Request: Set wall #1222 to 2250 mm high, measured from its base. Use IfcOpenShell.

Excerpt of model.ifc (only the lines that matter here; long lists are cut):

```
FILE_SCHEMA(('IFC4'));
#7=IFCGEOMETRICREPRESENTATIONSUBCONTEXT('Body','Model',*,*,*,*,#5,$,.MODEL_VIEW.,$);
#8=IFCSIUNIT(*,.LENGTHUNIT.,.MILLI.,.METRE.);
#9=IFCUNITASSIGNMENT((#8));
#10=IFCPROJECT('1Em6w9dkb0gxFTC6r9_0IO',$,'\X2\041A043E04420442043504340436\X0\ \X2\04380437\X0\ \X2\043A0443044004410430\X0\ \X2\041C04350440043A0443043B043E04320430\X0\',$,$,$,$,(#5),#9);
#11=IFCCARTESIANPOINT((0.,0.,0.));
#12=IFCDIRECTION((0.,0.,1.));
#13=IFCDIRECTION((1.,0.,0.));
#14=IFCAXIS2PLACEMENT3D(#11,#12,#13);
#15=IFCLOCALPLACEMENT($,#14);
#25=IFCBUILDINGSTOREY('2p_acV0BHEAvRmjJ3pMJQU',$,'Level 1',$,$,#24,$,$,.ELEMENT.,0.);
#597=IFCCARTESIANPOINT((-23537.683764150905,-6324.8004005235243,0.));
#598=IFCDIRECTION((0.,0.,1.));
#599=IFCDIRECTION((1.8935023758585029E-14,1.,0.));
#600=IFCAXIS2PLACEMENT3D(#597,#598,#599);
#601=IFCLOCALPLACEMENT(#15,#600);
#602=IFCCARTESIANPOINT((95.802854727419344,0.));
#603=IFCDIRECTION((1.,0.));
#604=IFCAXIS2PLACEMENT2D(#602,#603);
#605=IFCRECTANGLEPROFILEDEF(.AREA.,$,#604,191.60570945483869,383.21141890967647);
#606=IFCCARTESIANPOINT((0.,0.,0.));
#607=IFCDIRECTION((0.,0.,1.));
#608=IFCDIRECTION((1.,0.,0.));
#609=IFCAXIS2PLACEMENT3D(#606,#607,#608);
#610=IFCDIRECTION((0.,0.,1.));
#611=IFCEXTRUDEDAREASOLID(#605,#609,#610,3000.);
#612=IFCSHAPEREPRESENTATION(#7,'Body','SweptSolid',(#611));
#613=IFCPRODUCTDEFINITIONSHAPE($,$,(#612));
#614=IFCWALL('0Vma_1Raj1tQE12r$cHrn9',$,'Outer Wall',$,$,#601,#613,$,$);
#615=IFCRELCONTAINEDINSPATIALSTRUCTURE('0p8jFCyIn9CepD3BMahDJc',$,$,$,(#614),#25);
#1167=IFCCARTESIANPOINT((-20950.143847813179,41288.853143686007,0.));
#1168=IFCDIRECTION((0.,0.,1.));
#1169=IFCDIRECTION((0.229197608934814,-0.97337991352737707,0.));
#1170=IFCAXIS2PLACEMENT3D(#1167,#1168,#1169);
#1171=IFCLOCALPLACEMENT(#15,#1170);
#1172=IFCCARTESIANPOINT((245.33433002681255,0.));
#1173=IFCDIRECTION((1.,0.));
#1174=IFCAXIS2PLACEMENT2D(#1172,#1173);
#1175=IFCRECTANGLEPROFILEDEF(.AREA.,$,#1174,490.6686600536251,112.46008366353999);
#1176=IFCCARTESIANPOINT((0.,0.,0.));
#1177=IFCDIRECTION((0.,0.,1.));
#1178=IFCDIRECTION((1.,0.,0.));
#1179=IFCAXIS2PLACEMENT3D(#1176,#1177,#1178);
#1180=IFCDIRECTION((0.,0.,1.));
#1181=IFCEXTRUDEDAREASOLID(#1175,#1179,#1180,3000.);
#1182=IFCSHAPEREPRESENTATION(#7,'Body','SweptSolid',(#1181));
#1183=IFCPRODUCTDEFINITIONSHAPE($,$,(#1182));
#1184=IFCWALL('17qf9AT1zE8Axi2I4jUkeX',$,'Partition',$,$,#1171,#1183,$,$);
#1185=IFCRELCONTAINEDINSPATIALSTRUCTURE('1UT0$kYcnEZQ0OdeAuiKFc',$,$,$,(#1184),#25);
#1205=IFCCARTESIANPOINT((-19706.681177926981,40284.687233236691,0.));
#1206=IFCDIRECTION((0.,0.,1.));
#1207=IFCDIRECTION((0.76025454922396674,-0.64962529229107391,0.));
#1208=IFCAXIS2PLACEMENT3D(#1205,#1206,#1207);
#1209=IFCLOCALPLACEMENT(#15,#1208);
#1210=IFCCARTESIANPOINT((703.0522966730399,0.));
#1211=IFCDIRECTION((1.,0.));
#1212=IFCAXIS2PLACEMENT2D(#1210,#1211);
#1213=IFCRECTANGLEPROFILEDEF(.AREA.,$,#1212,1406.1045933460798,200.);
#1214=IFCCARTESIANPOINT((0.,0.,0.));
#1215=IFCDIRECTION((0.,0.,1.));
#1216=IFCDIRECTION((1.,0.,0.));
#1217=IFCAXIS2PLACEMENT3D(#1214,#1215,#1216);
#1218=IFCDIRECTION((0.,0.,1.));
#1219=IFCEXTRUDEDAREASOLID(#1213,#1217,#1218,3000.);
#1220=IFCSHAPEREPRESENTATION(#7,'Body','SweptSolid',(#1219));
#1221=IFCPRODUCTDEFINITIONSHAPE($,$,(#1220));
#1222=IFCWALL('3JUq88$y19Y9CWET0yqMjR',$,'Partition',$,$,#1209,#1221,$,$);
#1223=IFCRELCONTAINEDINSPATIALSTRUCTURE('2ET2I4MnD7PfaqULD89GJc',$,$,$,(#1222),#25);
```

```python
import ifcopenshell
import ifcopenshell.geom
import ifcopenshell.util.representation
import ifcopenshell.util.shape
import ifcopenshell.util.unit

model = ifcopenshell.open("model.ifc")
unit_scale = ifcopenshell.util.unit.calculate_unit_scale(model)
settings = ifcopenshell.geom.settings()


def volume(element):
    """Net volume in cubic metres, openings subtracted."""
    shape = ifcopenshell.geom.create_shape(settings, element)
    return ifcopenshell.util.shape.get_volume(shape.geometry)


wall = model.by_guid("3JUq88$y19Y9CWET0yqMjR")
before = volume(wall)

body = ifcopenshell.util.representation.get_representation(wall, "Model", "Body")
solid = body.Items[0]
old_height = solid.Depth
solid.Depth = 2.25 / unit_scale
after = volume(wall)

print(f"height {old_height:g} -> {solid.Depth:g}, volume {before:.3f} -> {after:.3f} m3")

model.write("model_v2.ifc")
```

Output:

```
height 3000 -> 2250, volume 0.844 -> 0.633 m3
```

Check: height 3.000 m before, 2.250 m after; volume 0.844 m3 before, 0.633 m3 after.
